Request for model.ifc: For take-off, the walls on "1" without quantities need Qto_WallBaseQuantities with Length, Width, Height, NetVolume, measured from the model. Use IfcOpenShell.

First a look at what the model holds.

```python
import ifcopenshell
import ifcopenshell.util.element
import ifcopenshell.util.unit

model = ifcopenshell.open("model.ifc")
print(model.schema)
for unit_type in ("LENGTHUNIT", "AREAUNIT", "VOLUMEUNIT"):
    print(unit_type, ifcopenshell.util.unit.calculate_unit_scale(model, unit_type))
storey = next(s for s in model.by_type("IfcBuildingStorey") if s.Name == "1")
walls = [e for e in ifcopenshell.util.element.get_decomposition(storey) if e.is_a("IfcWall")]
for e in sorted(walls, key=lambda e: e.id()):
    print(e.id(), e.is_a(), e.Name, list(ifcopenshell.util.element.get_psets(e, qtos_only=True)), sep=" | ")
```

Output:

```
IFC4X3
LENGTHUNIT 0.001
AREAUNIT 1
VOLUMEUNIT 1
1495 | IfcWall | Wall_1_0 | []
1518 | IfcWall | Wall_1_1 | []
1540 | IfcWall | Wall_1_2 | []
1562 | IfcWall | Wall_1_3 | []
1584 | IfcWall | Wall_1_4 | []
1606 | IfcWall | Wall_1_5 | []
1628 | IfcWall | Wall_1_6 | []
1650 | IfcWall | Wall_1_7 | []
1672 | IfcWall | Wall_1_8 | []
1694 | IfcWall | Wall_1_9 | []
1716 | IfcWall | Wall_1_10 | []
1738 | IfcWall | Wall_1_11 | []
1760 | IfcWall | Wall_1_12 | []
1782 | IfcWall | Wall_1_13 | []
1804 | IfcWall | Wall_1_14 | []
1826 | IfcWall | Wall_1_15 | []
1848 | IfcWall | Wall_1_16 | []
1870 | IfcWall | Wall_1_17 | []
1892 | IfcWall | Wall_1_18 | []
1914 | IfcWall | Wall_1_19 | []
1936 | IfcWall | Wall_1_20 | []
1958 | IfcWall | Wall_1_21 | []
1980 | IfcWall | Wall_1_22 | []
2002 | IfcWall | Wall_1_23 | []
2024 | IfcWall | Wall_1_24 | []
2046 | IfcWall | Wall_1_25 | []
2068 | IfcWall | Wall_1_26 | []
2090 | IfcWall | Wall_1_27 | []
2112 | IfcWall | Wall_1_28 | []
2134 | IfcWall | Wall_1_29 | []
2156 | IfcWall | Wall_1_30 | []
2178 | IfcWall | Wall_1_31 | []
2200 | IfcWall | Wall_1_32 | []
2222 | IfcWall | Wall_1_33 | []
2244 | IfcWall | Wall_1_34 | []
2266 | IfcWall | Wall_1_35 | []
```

```python
import ifcopenshell
import ifcopenshell.api.pset
import ifcopenshell.geom
import ifcopenshell.util.element
import ifcopenshell.util.shape
import ifcopenshell.util.unit

model = ifcopenshell.open("model.ifc")
unit_scale = ifcopenshell.util.unit.calculate_unit_scale(model)
volume_scale = ifcopenshell.util.unit.calculate_unit_scale(model, "VOLUMEUNIT")
settings = ifcopenshell.geom.settings()

storey = next(s for s in model.by_type("IfcBuildingStorey") if s.Name == "1")
walls = [e for e in ifcopenshell.util.element.get_decomposition(storey) if e.is_a("IfcWall")]

for e in sorted(walls, key=lambda e: e.id()):
    if ifcopenshell.util.element.get_psets(e, qtos_only=True, should_inherit=False):
        continue
    # Geometry comes back in metres, in the element's own axes.
    shape = ifcopenshell.geom.create_shape(settings, e)
    values = {
        "Length": ifcopenshell.util.shape.get_x(shape.geometry) / unit_scale,
        "Width": ifcopenshell.util.shape.get_y(shape.geometry) / unit_scale,
        "Height": ifcopenshell.util.shape.get_z(shape.geometry) / unit_scale,
        "NetVolume": ifcopenshell.util.shape.get_volume(shape.geometry) / volume_scale,
    }
    qto = ifcopenshell.api.pset.add_qto(model, product=e, name="Qto_WallBaseQuantities")
    ifcopenshell.api.pset.edit_qto(model, qto=qto, properties=values)
    print(e.id(), {k: round(v, 3) for k, v in values.items()})

model.write("model_v2.ifc")
```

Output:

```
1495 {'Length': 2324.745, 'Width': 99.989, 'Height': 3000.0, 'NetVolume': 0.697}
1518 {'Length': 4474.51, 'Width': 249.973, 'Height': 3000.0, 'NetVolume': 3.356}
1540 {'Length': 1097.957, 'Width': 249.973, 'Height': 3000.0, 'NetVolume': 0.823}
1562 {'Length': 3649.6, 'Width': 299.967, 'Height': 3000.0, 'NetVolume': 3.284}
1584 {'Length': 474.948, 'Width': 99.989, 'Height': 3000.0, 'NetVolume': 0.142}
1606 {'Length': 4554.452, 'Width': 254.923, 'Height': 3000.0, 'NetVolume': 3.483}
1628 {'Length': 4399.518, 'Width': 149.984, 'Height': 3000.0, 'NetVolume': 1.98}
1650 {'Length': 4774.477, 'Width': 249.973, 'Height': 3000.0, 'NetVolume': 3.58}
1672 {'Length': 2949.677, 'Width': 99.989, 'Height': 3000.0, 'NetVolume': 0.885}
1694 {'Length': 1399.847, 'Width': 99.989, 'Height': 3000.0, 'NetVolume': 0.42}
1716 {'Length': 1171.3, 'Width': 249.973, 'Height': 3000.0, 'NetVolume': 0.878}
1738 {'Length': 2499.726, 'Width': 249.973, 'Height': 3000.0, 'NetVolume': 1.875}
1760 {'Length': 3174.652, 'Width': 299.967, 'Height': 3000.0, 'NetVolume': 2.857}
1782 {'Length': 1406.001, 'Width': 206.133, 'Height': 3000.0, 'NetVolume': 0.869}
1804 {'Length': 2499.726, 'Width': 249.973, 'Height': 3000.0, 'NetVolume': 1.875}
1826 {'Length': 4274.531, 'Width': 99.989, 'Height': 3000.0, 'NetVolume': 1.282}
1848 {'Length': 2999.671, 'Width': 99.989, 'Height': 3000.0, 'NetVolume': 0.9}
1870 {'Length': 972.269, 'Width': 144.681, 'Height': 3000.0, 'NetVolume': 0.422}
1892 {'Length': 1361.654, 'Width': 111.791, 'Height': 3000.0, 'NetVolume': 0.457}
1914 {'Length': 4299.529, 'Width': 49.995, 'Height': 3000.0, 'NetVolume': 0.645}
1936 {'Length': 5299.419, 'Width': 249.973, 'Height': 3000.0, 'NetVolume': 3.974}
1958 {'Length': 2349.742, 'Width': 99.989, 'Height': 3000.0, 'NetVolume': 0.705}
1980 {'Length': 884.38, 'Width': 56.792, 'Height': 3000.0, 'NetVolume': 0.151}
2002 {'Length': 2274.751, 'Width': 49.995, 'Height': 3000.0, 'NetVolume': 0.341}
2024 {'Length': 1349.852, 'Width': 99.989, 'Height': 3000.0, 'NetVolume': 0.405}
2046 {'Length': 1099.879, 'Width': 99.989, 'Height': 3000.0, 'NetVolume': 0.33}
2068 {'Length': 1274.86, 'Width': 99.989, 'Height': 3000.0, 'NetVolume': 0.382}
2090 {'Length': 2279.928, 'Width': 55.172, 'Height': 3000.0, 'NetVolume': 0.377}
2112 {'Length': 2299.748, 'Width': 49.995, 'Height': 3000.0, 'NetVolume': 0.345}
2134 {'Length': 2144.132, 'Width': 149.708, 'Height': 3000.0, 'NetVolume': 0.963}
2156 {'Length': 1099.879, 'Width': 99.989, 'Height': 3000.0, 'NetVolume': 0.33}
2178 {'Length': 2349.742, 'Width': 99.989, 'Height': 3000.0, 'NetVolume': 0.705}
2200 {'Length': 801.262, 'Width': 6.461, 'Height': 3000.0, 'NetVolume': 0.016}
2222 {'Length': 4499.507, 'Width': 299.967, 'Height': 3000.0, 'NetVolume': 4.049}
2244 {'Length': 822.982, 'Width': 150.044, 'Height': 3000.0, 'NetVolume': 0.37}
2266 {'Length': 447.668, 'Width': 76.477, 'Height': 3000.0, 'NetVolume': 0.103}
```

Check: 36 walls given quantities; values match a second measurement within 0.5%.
